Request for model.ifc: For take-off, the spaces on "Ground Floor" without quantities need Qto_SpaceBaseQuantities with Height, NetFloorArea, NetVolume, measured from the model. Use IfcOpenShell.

First a look at what the model holds.

```python
import ifcopenshell
import ifcopenshell.util.element
import ifcopenshell.util.unit

model = ifcopenshell.open("model.ifc")
print(model.schema)
for unit_type in ("LENGTHUNIT", "AREAUNIT", "VOLUMEUNIT"):
    print(unit_type, ifcopenshell.util.unit.calculate_unit_scale(model, unit_type))
storey = next(s for s in model.by_type("IfcBuildingStorey") if s.Name == "Ground Floor")
spaces = [e for e in ifcopenshell.util.element.get_decomposition(storey) if e.is_a("IfcSpace")]
for e in sorted(spaces, key=lambda e: e.id()):
    print(e.id(), e.is_a(), e.Name, list(ifcopenshell.util.element.get_psets(e, qtos_only=True)), sep=" | ")
```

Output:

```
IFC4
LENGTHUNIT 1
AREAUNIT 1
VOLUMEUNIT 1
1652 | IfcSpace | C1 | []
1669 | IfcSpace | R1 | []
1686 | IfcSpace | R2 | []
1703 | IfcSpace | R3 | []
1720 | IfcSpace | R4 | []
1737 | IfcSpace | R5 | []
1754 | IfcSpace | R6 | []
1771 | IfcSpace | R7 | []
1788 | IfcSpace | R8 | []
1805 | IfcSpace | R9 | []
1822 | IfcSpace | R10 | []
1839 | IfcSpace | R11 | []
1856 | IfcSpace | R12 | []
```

```python
import ifcopenshell
import ifcopenshell.api.pset
import ifcopenshell.geom
import ifcopenshell.util.element
import ifcopenshell.util.shape
import ifcopenshell.util.unit

model = ifcopenshell.open("model.ifc")
unit_scale = ifcopenshell.util.unit.calculate_unit_scale(model)
area_scale = ifcopenshell.util.unit.calculate_unit_scale(model, "AREAUNIT")
volume_scale = ifcopenshell.util.unit.calculate_unit_scale(model, "VOLUMEUNIT")
settings = ifcopenshell.geom.settings()

storey = next(s for s in model.by_type("IfcBuildingStorey") if s.Name == "Ground Floor")
spaces = [e for e in ifcopenshell.util.element.get_decomposition(storey) if e.is_a("IfcSpace")]

for e in sorted(spaces, key=lambda e: e.id()):
    if ifcopenshell.util.element.get_psets(e, qtos_only=True, should_inherit=False):
        continue
    # Geometry comes back in metres, in the element's own axes.
    shape = ifcopenshell.geom.create_shape(settings, e)
    values = {
        "Height": ifcopenshell.util.shape.get_z(shape.geometry) / unit_scale,
        "NetFloorArea": ifcopenshell.util.shape.get_footprint_area(shape.geometry) / area_scale,
        "NetVolume": ifcopenshell.util.shape.get_volume(shape.geometry) / volume_scale,
    }
    qto = ifcopenshell.api.pset.add_qto(model, product=e, name="Qto_SpaceBaseQuantities")
    ifcopenshell.api.pset.edit_qto(model, qto=qto, properties=values)
    print(e.id(), {k: round(v, 3) for k, v in values.items()})

model.write("model_rev.ifc")
```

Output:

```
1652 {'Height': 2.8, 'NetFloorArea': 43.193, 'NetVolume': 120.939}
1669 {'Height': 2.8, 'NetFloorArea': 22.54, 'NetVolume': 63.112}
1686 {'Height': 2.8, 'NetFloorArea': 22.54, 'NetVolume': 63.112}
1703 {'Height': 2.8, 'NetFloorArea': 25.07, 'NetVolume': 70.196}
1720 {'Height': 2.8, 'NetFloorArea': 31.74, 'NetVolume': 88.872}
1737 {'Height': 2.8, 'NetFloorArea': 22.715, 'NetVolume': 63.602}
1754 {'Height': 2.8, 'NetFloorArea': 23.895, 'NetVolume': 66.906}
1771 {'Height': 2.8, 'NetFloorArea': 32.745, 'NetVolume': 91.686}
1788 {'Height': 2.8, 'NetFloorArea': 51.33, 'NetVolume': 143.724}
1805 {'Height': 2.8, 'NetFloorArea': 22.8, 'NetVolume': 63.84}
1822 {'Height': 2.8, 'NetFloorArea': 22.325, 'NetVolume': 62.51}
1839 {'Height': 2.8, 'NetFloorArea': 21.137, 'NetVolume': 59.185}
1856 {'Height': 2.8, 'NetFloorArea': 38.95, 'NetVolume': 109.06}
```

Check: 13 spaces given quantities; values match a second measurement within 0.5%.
